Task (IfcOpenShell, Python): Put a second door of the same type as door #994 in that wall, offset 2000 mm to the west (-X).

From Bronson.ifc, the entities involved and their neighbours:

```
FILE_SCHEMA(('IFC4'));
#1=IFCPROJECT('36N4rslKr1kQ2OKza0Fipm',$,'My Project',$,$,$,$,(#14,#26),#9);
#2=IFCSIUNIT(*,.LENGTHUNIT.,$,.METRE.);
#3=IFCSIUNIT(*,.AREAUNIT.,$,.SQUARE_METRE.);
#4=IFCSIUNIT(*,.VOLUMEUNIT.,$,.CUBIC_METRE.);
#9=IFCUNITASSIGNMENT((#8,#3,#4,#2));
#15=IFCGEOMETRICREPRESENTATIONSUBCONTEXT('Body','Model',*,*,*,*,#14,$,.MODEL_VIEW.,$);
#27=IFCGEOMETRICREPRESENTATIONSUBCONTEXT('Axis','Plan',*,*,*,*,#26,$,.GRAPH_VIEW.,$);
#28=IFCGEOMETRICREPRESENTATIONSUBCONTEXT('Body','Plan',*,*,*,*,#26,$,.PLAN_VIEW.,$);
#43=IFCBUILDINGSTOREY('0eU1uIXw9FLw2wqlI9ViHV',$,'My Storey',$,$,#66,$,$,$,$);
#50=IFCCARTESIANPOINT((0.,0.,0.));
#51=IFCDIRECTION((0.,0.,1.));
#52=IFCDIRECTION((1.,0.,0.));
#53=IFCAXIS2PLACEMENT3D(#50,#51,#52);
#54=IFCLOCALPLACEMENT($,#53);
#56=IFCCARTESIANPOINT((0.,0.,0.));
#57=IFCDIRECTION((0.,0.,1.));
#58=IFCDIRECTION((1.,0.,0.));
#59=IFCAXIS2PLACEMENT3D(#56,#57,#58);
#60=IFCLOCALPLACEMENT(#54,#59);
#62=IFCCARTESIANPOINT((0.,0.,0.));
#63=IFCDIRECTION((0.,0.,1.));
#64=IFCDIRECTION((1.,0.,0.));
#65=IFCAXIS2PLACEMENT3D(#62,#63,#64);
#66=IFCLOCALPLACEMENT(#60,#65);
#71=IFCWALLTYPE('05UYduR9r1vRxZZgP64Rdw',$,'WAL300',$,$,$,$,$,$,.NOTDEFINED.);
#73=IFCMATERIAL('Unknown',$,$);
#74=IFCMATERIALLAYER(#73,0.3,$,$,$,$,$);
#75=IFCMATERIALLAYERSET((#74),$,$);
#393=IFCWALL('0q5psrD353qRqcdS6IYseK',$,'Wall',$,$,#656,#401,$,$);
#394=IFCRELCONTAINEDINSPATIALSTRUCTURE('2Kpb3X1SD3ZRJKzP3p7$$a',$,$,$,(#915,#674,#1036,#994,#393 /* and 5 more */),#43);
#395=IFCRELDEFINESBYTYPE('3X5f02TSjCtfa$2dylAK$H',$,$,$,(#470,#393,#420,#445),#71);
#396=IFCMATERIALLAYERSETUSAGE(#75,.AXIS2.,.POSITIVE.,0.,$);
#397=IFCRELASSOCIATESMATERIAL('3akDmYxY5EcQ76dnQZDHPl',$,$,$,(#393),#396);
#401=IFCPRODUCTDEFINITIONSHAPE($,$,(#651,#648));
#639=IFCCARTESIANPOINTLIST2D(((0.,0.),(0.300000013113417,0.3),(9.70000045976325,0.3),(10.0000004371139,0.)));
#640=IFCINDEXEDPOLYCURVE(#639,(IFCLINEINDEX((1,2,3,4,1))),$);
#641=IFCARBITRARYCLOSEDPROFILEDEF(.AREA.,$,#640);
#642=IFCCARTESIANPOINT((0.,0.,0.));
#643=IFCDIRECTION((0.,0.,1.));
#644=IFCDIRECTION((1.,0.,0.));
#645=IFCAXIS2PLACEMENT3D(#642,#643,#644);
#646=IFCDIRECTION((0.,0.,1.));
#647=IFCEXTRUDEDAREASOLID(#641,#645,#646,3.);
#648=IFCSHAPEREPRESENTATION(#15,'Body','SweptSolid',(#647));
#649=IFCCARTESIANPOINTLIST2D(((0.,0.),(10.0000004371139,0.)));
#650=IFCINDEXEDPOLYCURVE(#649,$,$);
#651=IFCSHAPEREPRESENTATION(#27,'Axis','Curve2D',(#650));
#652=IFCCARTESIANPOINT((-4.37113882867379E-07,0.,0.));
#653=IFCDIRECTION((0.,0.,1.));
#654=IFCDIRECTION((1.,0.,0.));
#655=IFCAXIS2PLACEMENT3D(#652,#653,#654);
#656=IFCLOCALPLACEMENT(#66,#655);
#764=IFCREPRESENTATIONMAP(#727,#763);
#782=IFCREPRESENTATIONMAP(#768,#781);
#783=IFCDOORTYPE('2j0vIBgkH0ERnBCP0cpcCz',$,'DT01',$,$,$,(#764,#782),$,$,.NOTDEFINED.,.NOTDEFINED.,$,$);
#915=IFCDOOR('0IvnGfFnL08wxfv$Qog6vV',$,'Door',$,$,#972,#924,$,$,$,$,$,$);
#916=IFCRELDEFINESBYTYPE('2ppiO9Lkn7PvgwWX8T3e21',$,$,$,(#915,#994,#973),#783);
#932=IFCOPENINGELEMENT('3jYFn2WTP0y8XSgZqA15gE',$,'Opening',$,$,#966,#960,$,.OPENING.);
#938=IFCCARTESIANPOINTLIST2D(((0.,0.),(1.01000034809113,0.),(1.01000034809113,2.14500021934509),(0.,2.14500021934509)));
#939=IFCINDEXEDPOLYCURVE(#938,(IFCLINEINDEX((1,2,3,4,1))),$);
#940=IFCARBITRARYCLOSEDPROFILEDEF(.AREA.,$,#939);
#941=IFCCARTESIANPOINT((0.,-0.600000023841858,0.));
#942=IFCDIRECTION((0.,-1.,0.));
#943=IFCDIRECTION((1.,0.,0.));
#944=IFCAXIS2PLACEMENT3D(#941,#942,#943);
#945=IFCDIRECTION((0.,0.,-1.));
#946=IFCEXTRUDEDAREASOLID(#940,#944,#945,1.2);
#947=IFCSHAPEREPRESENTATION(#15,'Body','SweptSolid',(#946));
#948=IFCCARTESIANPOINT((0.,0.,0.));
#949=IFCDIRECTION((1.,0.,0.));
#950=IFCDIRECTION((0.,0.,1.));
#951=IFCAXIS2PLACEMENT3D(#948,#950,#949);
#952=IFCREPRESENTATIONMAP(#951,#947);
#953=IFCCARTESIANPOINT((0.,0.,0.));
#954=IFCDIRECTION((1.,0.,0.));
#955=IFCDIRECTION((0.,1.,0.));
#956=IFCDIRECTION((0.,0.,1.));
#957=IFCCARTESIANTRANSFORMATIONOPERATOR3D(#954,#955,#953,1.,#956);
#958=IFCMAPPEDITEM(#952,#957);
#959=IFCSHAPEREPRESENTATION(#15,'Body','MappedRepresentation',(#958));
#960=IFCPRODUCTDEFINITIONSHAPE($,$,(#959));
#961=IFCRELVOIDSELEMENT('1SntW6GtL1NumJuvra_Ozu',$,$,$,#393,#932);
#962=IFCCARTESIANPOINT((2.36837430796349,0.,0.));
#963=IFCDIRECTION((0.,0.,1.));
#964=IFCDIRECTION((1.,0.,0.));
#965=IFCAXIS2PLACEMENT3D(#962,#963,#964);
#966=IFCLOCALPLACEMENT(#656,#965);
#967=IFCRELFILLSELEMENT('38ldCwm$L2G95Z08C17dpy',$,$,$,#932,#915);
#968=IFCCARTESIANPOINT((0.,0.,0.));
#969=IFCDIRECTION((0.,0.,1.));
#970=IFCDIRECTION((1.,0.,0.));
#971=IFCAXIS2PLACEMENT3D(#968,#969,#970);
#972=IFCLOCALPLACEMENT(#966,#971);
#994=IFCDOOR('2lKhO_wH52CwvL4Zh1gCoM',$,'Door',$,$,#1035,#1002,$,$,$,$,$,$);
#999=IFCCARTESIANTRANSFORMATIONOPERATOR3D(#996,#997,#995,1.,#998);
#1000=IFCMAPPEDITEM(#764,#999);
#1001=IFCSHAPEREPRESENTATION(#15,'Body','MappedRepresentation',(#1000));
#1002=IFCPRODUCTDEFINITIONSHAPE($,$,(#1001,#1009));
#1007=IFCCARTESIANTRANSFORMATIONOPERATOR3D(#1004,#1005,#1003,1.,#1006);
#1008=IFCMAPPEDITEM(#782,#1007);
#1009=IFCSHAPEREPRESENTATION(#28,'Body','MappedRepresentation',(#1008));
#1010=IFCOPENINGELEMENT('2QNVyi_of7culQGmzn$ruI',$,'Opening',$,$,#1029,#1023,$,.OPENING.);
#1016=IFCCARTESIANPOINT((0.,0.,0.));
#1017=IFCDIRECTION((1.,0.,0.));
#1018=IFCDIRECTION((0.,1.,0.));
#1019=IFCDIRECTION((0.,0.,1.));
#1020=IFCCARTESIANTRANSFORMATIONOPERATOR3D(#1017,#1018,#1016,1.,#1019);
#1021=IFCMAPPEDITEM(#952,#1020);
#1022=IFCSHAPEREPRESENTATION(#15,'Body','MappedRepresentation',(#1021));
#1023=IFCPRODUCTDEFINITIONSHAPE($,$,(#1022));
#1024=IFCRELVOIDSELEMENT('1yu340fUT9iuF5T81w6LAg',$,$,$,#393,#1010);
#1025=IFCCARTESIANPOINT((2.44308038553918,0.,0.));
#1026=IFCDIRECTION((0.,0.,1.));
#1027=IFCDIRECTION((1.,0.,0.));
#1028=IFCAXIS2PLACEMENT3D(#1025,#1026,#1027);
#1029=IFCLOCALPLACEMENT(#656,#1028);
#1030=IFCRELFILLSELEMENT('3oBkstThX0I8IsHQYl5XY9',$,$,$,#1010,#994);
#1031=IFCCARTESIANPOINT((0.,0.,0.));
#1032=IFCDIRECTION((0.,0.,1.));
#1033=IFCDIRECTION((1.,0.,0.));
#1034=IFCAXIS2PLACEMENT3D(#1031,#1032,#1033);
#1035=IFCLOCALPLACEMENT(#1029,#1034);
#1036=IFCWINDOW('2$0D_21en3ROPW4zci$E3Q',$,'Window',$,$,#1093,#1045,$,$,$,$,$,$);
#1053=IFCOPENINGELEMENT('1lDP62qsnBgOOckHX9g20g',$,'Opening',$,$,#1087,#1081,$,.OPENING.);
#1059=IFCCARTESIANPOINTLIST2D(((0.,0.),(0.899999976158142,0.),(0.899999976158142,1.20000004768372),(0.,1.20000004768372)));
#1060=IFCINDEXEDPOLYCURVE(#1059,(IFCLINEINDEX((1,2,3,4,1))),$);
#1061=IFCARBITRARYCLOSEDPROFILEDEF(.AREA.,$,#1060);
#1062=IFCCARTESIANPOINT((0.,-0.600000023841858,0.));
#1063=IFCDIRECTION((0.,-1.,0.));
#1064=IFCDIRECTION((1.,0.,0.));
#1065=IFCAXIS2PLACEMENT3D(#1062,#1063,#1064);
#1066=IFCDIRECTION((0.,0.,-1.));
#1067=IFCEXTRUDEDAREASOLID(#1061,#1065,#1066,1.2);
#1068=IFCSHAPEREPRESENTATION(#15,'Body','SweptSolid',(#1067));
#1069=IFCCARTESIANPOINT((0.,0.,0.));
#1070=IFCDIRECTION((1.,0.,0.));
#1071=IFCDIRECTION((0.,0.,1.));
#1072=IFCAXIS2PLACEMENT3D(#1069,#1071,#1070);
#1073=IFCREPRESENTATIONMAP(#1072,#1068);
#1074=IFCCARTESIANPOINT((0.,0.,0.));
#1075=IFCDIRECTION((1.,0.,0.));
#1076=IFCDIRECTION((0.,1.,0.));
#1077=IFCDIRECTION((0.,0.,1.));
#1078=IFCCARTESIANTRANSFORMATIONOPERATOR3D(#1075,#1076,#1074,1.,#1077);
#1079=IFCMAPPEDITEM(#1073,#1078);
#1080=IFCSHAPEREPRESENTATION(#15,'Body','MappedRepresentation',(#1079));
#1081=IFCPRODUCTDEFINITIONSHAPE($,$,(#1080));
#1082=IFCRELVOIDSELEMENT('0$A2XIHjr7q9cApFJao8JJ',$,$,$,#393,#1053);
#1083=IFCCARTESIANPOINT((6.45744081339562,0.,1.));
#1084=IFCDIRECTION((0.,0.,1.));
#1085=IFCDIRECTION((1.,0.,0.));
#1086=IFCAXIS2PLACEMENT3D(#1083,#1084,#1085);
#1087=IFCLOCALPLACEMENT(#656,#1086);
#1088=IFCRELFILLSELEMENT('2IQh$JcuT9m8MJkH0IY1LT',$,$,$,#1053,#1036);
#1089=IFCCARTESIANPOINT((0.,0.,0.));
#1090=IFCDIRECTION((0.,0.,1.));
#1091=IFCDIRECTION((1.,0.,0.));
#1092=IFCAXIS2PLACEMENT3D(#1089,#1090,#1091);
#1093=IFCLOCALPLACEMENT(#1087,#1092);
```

```python
import ifcopenshell
import ifcopenshell.api.feature
import ifcopenshell.api.geometry
import ifcopenshell.api.root
import ifcopenshell.geom
import ifcopenshell.util.element
import ifcopenshell.util.placement
import ifcopenshell.util.shape
import ifcopenshell.util.unit

model = ifcopenshell.open("Bronson.ifc")
unit_scale = ifcopenshell.util.unit.calculate_unit_scale(model)
settings = ifcopenshell.geom.settings()


def volume(element):
    """Net volume in cubic metres, openings subtracted."""
    shape = ifcopenshell.geom.create_shape(settings, element)
    return ifcopenshell.util.shape.get_volume(shape.geometry)


door = model.by_guid("2lKhO_wH52CwvL4Zh1gCoM")
opening = door.FillsVoids[0].RelatingOpeningElement
wall = opening.VoidsElements[0].RelatingBuildingElement
before = volume(wall)
shift = ifcopenshell.util.placement.get_local_placement(wall.ObjectPlacement)[:3, 0] * -2 / unit_scale

# copy_class copies the void relationship, type, container and properties, but no geometry.
new_opening = ifcopenshell.api.root.copy_class(model, product=opening)
new_opening.Representation = ifcopenshell.util.element.copy_deep(
    model, opening.Representation, exclude=["IfcGeometricRepresentationContext", "IfcRepresentationMap"]
)
new_door = ifcopenshell.api.root.copy_class(model, product=door)
new_door.Representation = ifcopenshell.util.element.copy_deep(
    model, door.Representation, exclude=["IfcGeometricRepresentationContext", "IfcRepresentationMap"]
)
ifcopenshell.api.feature.add_filling(model, opening=new_opening, element=new_door)

for old, new in ((opening, new_opening), (door, new_door)):
    matrix = ifcopenshell.util.placement.get_local_placement(old.ObjectPlacement)
    matrix[:3, 3] += shift
    ifcopenshell.api.geometry.edit_object_placement(model, product=new, matrix=matrix, is_si=False)

after = volume(wall)

print(f"wall volume {before:.3f} -> {after:.3f} m3")

model.write("Bronson-out.ifc")
```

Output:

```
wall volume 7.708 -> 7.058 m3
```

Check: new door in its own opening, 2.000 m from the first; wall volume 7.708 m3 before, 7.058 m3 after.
